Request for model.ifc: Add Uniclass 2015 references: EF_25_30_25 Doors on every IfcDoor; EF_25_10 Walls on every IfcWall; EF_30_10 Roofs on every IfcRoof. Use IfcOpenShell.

First a look at what the model holds.

```python
import ifcopenshell

model = ifcopenshell.open("model.ifc")
print(model.schema)
print("classifications:", [c.Name for c in model.by_type("IfcClassification")])
for ifc_class in ("IfcDoor", "IfcRoof", "IfcStair", "IfcWall", "IfcWindow"):
    print(ifc_class, len(model.by_type(ifc_class)))
```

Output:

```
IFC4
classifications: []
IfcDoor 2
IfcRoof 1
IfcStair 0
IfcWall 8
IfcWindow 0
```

```python
import ifcopenshell
import ifcopenshell.api.classification

model = ifcopenshell.open("model.ifc")

system = ifcopenshell.api.classification.add_classification(model, classification="Uniclass 2015")

codes = {
    "IfcDoor": ("EF_25_30_25", "Doors"),
    "IfcWall": ("EF_25_10", "Walls"),
    "IfcRoof": ("EF_30_10", "Roofs"),
}
for ifc_class, (code, name) in codes.items():
    products = model.by_type(ifc_class)
    ifcopenshell.api.classification.add_reference(
        model, products=products, classification=system, identification=code, name=name
    )
    print(code, len(products))

model.write("model-out.ifc")
```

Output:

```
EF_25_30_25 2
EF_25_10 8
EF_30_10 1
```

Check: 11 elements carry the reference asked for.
